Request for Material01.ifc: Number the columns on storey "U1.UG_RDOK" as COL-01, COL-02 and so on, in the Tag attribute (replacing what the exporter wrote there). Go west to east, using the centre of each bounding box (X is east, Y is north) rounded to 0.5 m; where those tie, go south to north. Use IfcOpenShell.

First a look at what the model holds.

```python
import ifcopenshell
import ifcopenshell.util.element
import ifcopenshell.util.placement

model = ifcopenshell.open("Material01.ifc")
print(model.schema)
storey = next(s for s in model.by_type("IfcBuildingStorey") if s.Name == "U1.UG_RDOK")
columns = [e for e in ifcopenshell.util.element.get_decomposition(storey) if e.is_a("IfcColumn")]
for e in sorted(columns, key=lambda e: e.id()):
    origin = ifcopenshell.util.placement.get_local_placement(e.ObjectPlacement)[:3, 3]
    print(e.id(), e.Tag, e.Name, origin.round(2) + 0.0, sep=" | ")
```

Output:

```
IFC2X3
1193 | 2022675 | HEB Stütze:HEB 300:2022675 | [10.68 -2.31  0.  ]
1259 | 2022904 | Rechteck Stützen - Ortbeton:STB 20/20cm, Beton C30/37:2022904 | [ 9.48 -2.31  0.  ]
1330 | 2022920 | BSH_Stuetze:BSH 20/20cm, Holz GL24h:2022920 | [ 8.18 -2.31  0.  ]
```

```python
import ifcopenshell
import ifcopenshell.geom
import ifcopenshell.util.element
import ifcopenshell.util.shape

model = ifcopenshell.open("Material01.ifc")
settings = ifcopenshell.geom.settings()
settings.set("use-world-coords", True)


def centre(element):
    shape = ifcopenshell.geom.create_shape(settings, element)
    return ifcopenshell.util.shape.get_bbox_centroid(shape.geometry)


storey = next(s for s in model.by_type("IfcBuildingStorey") if s.Name == "U1.UG_RDOK")
columns = [e for e in ifcopenshell.util.element.get_decomposition(storey) if e.is_a("IfcColumn")]

# Insertion points can sit at a corner or the storey origin, so sort by the geometry (in metres).
centres = {e: centre(e) for e in columns}
columns.sort(key=lambda e: (round(centres[e][0] / 0.5), centres[e][1]))

for i, e in enumerate(columns, start=1):
    number = f"COL-{i:02d}"
    e.Tag = number
    print(e.id(), number)

model.write("Material01-out.ifc")
```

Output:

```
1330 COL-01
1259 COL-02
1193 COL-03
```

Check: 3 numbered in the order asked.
